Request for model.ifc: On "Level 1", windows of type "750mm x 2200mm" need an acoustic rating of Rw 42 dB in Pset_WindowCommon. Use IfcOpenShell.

First a look at what the model holds.

```python
import ifcopenshell
import ifcopenshell.util.element

model = ifcopenshell.open("model.ifc")
print(model.schema)
storey = next(s for s in model.by_type("IfcBuildingStorey") if s.Name == "Level 1")
windows = [e for e in ifcopenshell.util.element.get_decomposition(storey) if e.is_a("IfcWindow")]
seen = {}
for e in windows:
    element_type = ifcopenshell.util.element.get_type(e)
    key = (element_type.Name if element_type != e and element_type else None, ifcopenshell.util.element.get_pset(e, "Pset_WindowCommon", "AcousticRating"))
    seen[key] = seen.get(key, 0) + 1
for (name, value), count in sorted(seen.items(), key=str):
    print(count, "x", name, "|", value)
```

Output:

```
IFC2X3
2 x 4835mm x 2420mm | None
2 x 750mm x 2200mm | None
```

```python
import ifcopenshell
import ifcopenshell.api.pset
import ifcopenshell.util.element

model = ifcopenshell.open("model.ifc")

storey = next(s for s in model.by_type("IfcBuildingStorey") if s.Name == "Level 1")
windows = [e for e in ifcopenshell.util.element.get_decomposition(storey) if e.is_a("IfcWindow")]

count = 0
for e in windows:
    element_type = ifcopenshell.util.element.get_type(e)
    if element_type in (None, e) or element_type.Name != "750mm x 2200mm":
        continue
    # add_pset returns the element's existing set when there is one.
    pset = ifcopenshell.api.pset.add_pset(model, product=e, name="Pset_WindowCommon")
    ifcopenshell.api.pset.edit_pset(model, pset=pset, properties={"AcousticRating": "Rw 42 dB"})
    count += 1

print(count, "windows updated")

model.write("model-out.ifc")
```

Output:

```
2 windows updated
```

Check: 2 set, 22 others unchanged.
